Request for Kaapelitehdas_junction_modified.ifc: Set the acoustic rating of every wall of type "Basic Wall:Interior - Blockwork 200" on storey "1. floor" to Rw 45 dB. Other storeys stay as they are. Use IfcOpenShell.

First a look at what the model holds.

```python
import ifcopenshell
import ifcopenshell.util.element

model = ifcopenshell.open("Kaapelitehdas_junction_modified.ifc")
print(model.schema)
storey = next(s for s in model.by_type("IfcBuildingStorey") if s.Name == "1. floor")
walls = [e for e in ifcopenshell.util.element.get_decomposition(storey) if e.is_a("IfcWall")]
seen = {}
for e in walls:
    element_type = ifcopenshell.util.element.get_type(e)
    key = (element_type.Name if element_type != e and element_type else None, ifcopenshell.util.element.get_pset(e, "Pset_WallCommon", "AcousticRating"))
    seen[key] = seen.get(key, 0) + 1
for (name, value), count in sorted(seen.items(), key=str):
    print(count, "x", name, "|", value)
```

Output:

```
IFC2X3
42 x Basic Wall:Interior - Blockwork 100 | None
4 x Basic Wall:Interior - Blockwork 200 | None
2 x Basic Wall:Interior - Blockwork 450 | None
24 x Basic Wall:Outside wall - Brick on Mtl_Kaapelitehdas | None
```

```python
import ifcopenshell
import ifcopenshell.api.pset
import ifcopenshell.util.element

model = ifcopenshell.open("Kaapelitehdas_junction_modified.ifc")

storey = next(s for s in model.by_type("IfcBuildingStorey") if s.Name == "1. floor")
walls = [e for e in ifcopenshell.util.element.get_decomposition(storey) if e.is_a("IfcWall")]

count = 0
for e in walls:
    element_type = ifcopenshell.util.element.get_type(e)
    if element_type in (None, e) or element_type.Name != "Basic Wall:Interior - Blockwork 200":
        continue
    # add_pset returns the element's existing set when there is one.
    pset = ifcopenshell.api.pset.add_pset(model, product=e, name="Pset_WallCommon")
    ifcopenshell.api.pset.edit_pset(model, pset=pset, properties={"AcousticRating": "Rw 45 dB"})
    count += 1

print(count, "walls updated")

model.write("Kaapelitehdas_junction_modified-out.ifc")
```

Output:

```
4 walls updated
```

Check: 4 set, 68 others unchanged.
